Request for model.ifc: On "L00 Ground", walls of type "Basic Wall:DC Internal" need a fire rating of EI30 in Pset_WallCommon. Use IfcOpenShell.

First a look at what the model holds.

```python
import ifcopenshell
import ifcopenshell.util.element

model = ifcopenshell.open("model.ifc")
print(model.schema)
storey = next(s for s in model.by_type("IfcBuildingStorey") if s.Name == "L00 Ground")
walls = [e for e in ifcopenshell.util.element.get_decomposition(storey) if e.is_a("IfcWall")]
seen = {}
for e in walls:
    element_type = ifcopenshell.util.element.get_type(e)
    key = (element_type.Name if element_type != e and element_type else None, ifcopenshell.util.element.get_pset(e, "Pset_WallCommon", "FireRating"))
    seen[key] = seen.get(key, 0) + 1
for (name, value), count in sorted(seen.items(), key=str):
    print(count, "x", name, "|", value)
```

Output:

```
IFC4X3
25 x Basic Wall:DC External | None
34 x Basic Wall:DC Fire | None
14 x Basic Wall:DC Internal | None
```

```python
import ifcopenshell
import ifcopenshell.api.pset
import ifcopenshell.util.element

model = ifcopenshell.open("model.ifc")

storey = next(s for s in model.by_type("IfcBuildingStorey") if s.Name == "L00 Ground")
walls = [e for e in ifcopenshell.util.element.get_decomposition(storey) if e.is_a("IfcWall")]

count = 0
for e in walls:
    element_type = ifcopenshell.util.element.get_type(e)
    if element_type in (None, e) or element_type.Name != "Basic Wall:DC Internal":
        continue
    # add_pset returns the element's existing set when there is one.
    pset = ifcopenshell.api.pset.add_pset(model, product=e, name="Pset_WallCommon")
    ifcopenshell.api.pset.edit_pset(model, pset=pset, properties={"FireRating": "EI30"})
    count += 1

print(count, "walls updated")

model.write("model_rev.ifc")
```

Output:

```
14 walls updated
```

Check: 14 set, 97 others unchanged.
